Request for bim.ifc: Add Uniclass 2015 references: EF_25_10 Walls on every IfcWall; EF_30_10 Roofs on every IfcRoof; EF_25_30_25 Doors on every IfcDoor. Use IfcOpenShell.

First a look at what the model holds.

```python
import ifcopenshell

model = ifcopenshell.open("bim.ifc")
print(model.schema)
print("classifications:", [c.Name for c in model.by_type("IfcClassification")])
for ifc_class in ("IfcDoor", "IfcRoof", "IfcStair", "IfcWall", "IfcWindow"):
    print(ifc_class, len(model.by_type(ifc_class)))
```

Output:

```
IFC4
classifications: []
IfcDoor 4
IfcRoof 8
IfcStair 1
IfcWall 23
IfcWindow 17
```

```python
import ifcopenshell
import ifcopenshell.api.classification

model = ifcopenshell.open("bim.ifc")

system = ifcopenshell.api.classification.add_classification(model, classification="Uniclass 2015")

codes = {
    "IfcWall": ("EF_25_10", "Walls"),
    "IfcRoof": ("EF_30_10", "Roofs"),
    "IfcDoor": ("EF_25_30_25", "Doors"),
}
for ifc_class, (code, name) in codes.items():
    products = model.by_type(ifc_class)
    ifcopenshell.api.classification.add_reference(
        model, products=products, classification=system, identification=code, name=name
    )
    print(code, len(products))

model.write("bim_v2.ifc")
```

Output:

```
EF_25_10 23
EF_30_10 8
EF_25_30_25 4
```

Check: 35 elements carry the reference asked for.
